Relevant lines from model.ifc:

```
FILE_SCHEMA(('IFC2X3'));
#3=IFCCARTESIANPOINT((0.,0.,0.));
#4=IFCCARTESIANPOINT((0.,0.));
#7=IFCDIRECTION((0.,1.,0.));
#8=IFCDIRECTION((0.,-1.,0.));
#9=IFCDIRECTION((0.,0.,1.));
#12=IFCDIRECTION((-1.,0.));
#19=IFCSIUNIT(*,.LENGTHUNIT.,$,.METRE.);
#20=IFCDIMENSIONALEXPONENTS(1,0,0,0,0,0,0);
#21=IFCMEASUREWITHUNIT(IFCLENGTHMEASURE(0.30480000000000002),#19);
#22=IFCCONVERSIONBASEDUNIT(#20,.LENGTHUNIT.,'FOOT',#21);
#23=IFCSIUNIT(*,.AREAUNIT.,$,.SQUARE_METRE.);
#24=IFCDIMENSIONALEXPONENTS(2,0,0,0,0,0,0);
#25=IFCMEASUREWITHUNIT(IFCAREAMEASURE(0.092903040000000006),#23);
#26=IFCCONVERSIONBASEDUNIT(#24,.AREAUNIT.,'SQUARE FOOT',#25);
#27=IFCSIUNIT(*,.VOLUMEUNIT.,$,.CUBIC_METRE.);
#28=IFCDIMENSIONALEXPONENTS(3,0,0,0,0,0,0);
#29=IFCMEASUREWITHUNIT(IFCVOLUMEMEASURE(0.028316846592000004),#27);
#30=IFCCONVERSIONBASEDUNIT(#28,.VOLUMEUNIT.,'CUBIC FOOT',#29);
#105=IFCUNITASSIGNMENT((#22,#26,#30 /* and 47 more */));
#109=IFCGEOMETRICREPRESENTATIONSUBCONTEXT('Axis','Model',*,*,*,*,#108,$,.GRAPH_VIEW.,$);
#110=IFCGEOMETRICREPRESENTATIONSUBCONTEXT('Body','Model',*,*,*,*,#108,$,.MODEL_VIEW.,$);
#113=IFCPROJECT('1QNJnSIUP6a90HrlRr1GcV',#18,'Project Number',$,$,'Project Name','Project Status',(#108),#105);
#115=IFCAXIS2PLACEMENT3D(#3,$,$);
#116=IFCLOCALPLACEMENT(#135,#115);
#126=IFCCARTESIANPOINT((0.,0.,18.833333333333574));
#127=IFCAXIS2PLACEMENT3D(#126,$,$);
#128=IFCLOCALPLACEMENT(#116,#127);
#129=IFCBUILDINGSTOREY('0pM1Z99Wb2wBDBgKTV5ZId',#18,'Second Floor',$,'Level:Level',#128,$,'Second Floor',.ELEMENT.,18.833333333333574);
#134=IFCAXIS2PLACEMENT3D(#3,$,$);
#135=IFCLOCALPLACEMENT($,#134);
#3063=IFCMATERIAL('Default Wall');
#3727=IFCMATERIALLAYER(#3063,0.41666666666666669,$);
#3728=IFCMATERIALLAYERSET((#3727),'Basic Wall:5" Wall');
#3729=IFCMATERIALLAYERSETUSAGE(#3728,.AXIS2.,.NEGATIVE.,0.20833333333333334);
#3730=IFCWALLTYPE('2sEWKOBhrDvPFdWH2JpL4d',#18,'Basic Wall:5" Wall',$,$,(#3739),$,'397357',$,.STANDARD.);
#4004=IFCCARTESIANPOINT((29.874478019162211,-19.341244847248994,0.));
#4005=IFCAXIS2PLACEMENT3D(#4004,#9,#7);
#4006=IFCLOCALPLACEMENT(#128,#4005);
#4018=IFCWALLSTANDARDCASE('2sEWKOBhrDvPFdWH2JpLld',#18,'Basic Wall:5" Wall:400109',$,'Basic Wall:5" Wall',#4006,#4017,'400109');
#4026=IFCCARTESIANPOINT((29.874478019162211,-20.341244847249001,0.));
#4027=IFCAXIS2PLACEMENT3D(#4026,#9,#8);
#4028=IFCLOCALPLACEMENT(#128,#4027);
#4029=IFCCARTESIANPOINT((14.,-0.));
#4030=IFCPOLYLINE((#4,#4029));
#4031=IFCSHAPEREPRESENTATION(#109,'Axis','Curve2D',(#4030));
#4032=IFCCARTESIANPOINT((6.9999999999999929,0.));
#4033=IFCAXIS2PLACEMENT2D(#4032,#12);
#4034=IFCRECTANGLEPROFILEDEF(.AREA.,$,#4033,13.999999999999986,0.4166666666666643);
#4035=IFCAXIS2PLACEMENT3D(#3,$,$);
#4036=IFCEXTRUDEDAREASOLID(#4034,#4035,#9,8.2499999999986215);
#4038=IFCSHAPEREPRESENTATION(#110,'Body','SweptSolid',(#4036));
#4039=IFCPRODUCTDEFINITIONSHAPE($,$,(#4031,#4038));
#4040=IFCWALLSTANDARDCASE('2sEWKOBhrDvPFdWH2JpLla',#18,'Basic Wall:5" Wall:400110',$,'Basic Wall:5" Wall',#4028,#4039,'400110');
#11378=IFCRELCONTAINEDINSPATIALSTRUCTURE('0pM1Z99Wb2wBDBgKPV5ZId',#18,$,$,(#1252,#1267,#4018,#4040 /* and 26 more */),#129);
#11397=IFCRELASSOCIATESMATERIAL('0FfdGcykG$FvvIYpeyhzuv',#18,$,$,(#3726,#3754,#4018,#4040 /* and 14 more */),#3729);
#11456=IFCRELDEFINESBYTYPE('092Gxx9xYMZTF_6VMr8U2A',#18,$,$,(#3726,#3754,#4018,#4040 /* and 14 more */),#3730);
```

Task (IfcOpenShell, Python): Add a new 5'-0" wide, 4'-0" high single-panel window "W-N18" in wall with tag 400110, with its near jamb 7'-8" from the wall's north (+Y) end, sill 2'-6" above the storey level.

```python
import numpy as np
import ifcopenshell
import ifcopenshell.api.feature
import ifcopenshell.api.geometry
import ifcopenshell.api.root
import ifcopenshell.api.spatial
import ifcopenshell.api.type
import ifcopenshell.geom
import ifcopenshell.util.element
import ifcopenshell.util.placement
import ifcopenshell.util.representation
import ifcopenshell.util.shape
import ifcopenshell.util.unit

model = ifcopenshell.open("model.ifc")
unit_scale = ifcopenshell.util.unit.calculate_unit_scale(model)
settings = ifcopenshell.geom.settings()


def volume(element):
    """Net volume in cubic metres, openings subtracted."""
    shape = ifcopenshell.geom.create_shape(settings, element)
    return ifcopenshell.util.shape.get_volume(shape.geometry)


wall = model.by_id(4040)
storey = ifcopenshell.util.element.get_container(wall, ifc_class="IfcBuildingStorey")
context = ifcopenshell.util.representation.get_context(model, "Model", "Body", "MODEL_VIEW")
before = volume(wall)

width, height, from_end, sill = 1.524, 1.2192, 2.3368, 0.762  # metres

# The wall runs along its own X axis, and the end named is its -X end.
wall_shape = ifcopenshell.geom.create_shape(settings, wall)
x, y, z = ifcopenshell.util.shape.get_vertices(wall_shape.geometry).T
start = x.min() + from_end
face, thickness = float(y.min()), float(y.max() - y.min())
wall_matrix = ifcopenshell.util.placement.get_local_placement(wall.ObjectPlacement)
level = ifcopenshell.util.placement.get_local_placement(storey.ObjectPlacement)[2, 3]


def in_wall(x, y):
    """Placement at x, y metres in the wall's axes, at sill height."""
    matrix = wall_matrix.copy()
    matrix[:, 3] = wall_matrix @ np.array([x / unit_scale, y / unit_scale, 0.0, 1.0])
    matrix[2, 3] = level + sill / unit_scale
    return matrix


# Opening: a box that overshoots both wall faces by 50 mm.
opening = ifcopenshell.api.root.create_entity(model, ifc_class="IfcOpeningElement")
box = ifcopenshell.api.geometry.add_wall_representation(
    model, context=context, length=width, height=height, thickness=thickness + 0.1
)
ifcopenshell.api.geometry.assign_representation(model, product=opening, representation=box)
ifcopenshell.api.geometry.edit_object_placement(model, product=opening, matrix=in_wall(start, face - 0.05), is_si=False)
ifcopenshell.api.feature.add_feature(model, feature=opening, element=wall)

window = ifcopenshell.api.root.create_entity(model, ifc_class="IfcWindow", name="W-N18")
window.OverallWidth, window.OverallHeight = width / unit_scale, height / unit_scale
body = ifcopenshell.api.geometry.add_window_representation(
    model,
    context=context,
    overall_width=window.OverallWidth,
    overall_height=window.OverallHeight,
    partition_type="SINGLE_PANEL",
)
ifcopenshell.api.geometry.assign_representation(model, product=window, representation=body)
ifcopenshell.api.spatial.assign_container(model, products=[window], relating_structure=storey)
fills = ifcopenshell.api.feature.add_filling(model, opening=opening, element=window)
fills.OwnerHistory = window.OwnerHistory  # required in IFC2X3

# IFC2X3 keeps the operation on the window style.
style = ifcopenshell.api.root.create_entity(model, ifc_class="IfcWindowStyle", name="W-N18")
style.OperationType, style.ConstructionType = "SINGLE_PANEL", "NOTDEFINED"
style.ParameterTakesPrecedence = style.Sizeable = False
ifcopenshell.api.type.assign_type(model, related_objects=[window], relating_type=style)

# Centre the window in the wall's thickness.
ifcopenshell.api.geometry.edit_object_placement(model, product=window, matrix=in_wall(start, face), is_si=False)
window_shape = ifcopenshell.geom.create_shape(settings, window)
depth = ifcopenshell.util.shape.get_vertices(window_shape.geometry)[:, 1]
offset = face + thickness / 2 - (depth.min() + depth.max()) / 2
ifcopenshell.api.geometry.edit_object_placement(model, product=window, matrix=in_wall(start, offset), is_si=False)

after = volume(wall)

print(f"wall volume {before:.3f} -> {after:.3f} m3")

model.write("model_v2.ifc")
```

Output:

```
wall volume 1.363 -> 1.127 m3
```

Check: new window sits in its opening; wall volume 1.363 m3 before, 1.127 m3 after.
